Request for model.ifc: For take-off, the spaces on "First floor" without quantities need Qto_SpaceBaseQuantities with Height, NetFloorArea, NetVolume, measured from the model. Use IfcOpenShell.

First a look at what the model holds.

```python
import ifcopenshell
import ifcopenshell.util.element
import ifcopenshell.util.unit

model = ifcopenshell.open("model.ifc")
print(model.schema)
for unit_type in ("LENGTHUNIT", "AREAUNIT", "VOLUMEUNIT"):
    print(unit_type, ifcopenshell.util.unit.calculate_unit_scale(model, unit_type))
storey = next(s for s in model.by_type("IfcBuildingStorey") if s.Name == "First floor")
spaces = [e for e in ifcopenshell.util.element.get_decomposition(storey) if e.is_a("IfcSpace")]
for e in sorted(spaces, key=lambda e: e.id()):
    print(e.id(), e.is_a(), e.Name, list(ifcopenshell.util.element.get_psets(e, qtos_only=True)), sep=" | ")
```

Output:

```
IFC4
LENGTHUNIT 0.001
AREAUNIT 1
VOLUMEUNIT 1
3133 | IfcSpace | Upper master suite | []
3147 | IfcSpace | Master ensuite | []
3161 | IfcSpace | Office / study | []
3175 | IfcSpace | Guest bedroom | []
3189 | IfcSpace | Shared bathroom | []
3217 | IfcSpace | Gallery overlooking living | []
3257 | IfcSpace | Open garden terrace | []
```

```python
import ifcopenshell
import ifcopenshell.api.pset
import ifcopenshell.geom
import ifcopenshell.util.element
import ifcopenshell.util.shape
import ifcopenshell.util.unit

model = ifcopenshell.open("model.ifc")
unit_scale = ifcopenshell.util.unit.calculate_unit_scale(model)
area_scale = ifcopenshell.util.unit.calculate_unit_scale(model, "AREAUNIT")
volume_scale = ifcopenshell.util.unit.calculate_unit_scale(model, "VOLUMEUNIT")
settings = ifcopenshell.geom.settings()

storey = next(s for s in model.by_type("IfcBuildingStorey") if s.Name == "First floor")
spaces = [e for e in ifcopenshell.util.element.get_decomposition(storey) if e.is_a("IfcSpace")]

for e in sorted(spaces, key=lambda e: e.id()):
    if ifcopenshell.util.element.get_psets(e, qtos_only=True, should_inherit=False):
        continue
    # Geometry comes back in metres, in the element's own axes.
    shape = ifcopenshell.geom.create_shape(settings, e)
    values = {
        "Height": ifcopenshell.util.shape.get_z(shape.geometry) / unit_scale,
        "NetFloorArea": ifcopenshell.util.shape.get_footprint_area(shape.geometry) / area_scale,
        "NetVolume": ifcopenshell.util.shape.get_volume(shape.geometry) / volume_scale,
    }
    qto = ifcopenshell.api.pset.add_qto(model, product=e, name="Qto_SpaceBaseQuantities")
    ifcopenshell.api.pset.edit_qto(model, qto=qto, properties=values)
    print(e.id(), {k: round(v, 3) for k, v in values.items()})

model.write("model-out.ifc")
```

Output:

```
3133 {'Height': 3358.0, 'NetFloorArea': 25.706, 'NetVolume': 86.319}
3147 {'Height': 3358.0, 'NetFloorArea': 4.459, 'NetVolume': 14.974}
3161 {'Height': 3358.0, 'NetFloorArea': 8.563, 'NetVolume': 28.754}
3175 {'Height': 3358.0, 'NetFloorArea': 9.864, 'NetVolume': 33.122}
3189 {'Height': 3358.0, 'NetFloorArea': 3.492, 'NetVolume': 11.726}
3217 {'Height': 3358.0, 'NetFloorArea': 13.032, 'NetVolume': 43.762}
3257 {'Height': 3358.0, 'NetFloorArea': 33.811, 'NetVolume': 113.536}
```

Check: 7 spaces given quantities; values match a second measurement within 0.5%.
